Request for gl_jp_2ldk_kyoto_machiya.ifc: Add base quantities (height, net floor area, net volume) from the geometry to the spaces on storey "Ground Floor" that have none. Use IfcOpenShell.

First a look at what the model holds.

```python
import ifcopenshell
import ifcopenshell.util.element
import ifcopenshell.util.unit

model = ifcopenshell.open("gl_jp_2ldk_kyoto_machiya.ifc")
print(model.schema)
for unit_type in ("LENGTHUNIT", "AREAUNIT", "VOLUMEUNIT"):
    print(unit_type, ifcopenshell.util.unit.calculate_unit_scale(model, unit_type))
storey = next(s for s in model.by_type("IfcBuildingStorey") if s.Name == "Ground Floor")
spaces = [e for e in ifcopenshell.util.element.get_decomposition(storey) if e.is_a("IfcSpace")]
for e in sorted(spaces, key=lambda e: e.id()):
    print(e.id(), e.is_a(), e.Name, list(ifcopenshell.util.element.get_psets(e, qtos_only=True)), sep=" | ")
```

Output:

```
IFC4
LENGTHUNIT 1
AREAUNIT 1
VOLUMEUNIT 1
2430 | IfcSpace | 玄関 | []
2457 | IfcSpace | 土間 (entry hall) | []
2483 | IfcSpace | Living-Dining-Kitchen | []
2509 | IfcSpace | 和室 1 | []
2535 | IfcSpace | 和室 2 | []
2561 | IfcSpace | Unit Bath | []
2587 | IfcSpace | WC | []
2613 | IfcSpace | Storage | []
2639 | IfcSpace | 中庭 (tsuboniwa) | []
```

```python
import ifcopenshell
import ifcopenshell.api.pset
import ifcopenshell.geom
import ifcopenshell.util.element
import ifcopenshell.util.shape
import ifcopenshell.util.unit

model = ifcopenshell.open("gl_jp_2ldk_kyoto_machiya.ifc")
unit_scale = ifcopenshell.util.unit.calculate_unit_scale(model)
area_scale = ifcopenshell.util.unit.calculate_unit_scale(model, "AREAUNIT")
volume_scale = ifcopenshell.util.unit.calculate_unit_scale(model, "VOLUMEUNIT")
settings = ifcopenshell.geom.settings()

storey = next(s for s in model.by_type("IfcBuildingStorey") if s.Name == "Ground Floor")
spaces = [e for e in ifcopenshell.util.element.get_decomposition(storey) if e.is_a("IfcSpace")]

for e in sorted(spaces, key=lambda e: e.id()):
    if ifcopenshell.util.element.get_psets(e, qtos_only=True, should_inherit=False):
        continue
    # Geometry comes back in metres, in the element's own axes.
    shape = ifcopenshell.geom.create_shape(settings, e)
    values = {
        "Height": ifcopenshell.util.shape.get_z(shape.geometry) / unit_scale,
        "NetFloorArea": ifcopenshell.util.shape.get_footprint_area(shape.geometry) / area_scale,
        "NetVolume": ifcopenshell.util.shape.get_volume(shape.geometry) / volume_scale,
    }
    qto = ifcopenshell.api.pset.add_qto(model, product=e, name="Qto_SpaceBaseQuantities")
    ifcopenshell.api.pset.edit_qto(model, qto=qto, properties=values)
    print(e.id(), {k: round(v, 3) for k, v in values.items()})

model.write("gl_jp_2ldk_kyoto_machiya-out.ifc")
```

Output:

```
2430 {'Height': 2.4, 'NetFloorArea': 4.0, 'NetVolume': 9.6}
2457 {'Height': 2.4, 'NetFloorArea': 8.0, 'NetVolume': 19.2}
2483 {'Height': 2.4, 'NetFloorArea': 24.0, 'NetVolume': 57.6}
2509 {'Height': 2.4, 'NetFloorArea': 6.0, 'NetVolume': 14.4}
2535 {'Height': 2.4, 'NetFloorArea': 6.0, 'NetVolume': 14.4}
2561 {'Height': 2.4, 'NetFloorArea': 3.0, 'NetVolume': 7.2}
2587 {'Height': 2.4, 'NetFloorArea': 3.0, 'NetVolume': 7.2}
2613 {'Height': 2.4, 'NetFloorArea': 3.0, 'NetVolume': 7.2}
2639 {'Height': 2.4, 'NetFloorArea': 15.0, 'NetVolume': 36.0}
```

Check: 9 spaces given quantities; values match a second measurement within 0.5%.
